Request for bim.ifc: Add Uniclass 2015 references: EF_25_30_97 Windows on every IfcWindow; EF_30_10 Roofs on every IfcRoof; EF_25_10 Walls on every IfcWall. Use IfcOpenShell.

First a look at what the model holds.

```python
import ifcopenshell

model = ifcopenshell.open("bim.ifc")
print(model.schema)
print("classifications:", [c.Name for c in model.by_type("IfcClassification")])
for ifc_class in ("IfcDoor", "IfcRoof", "IfcStair", "IfcWall", "IfcWindow"):
    print(ifc_class, len(model.by_type(ifc_class)))
```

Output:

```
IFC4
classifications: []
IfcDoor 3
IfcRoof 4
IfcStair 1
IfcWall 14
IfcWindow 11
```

```python
import ifcopenshell
import ifcopenshell.api.classification

model = ifcopenshell.open("bim.ifc")

system = ifcopenshell.api.classification.add_classification(model, classification="Uniclass 2015")

codes = {
    "IfcWindow": ("EF_25_30_97", "Windows"),
    "IfcRoof": ("EF_30_10", "Roofs"),
    "IfcWall": ("EF_25_10", "Walls"),
}
for ifc_class, (code, name) in codes.items():
    products = model.by_type(ifc_class)
    ifcopenshell.api.classification.add_reference(
        model, products=products, classification=system, identification=code, name=name
    )
    print(code, len(products))

model.write("bim_rev.ifc")
```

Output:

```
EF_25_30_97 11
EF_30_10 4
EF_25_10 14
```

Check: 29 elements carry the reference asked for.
